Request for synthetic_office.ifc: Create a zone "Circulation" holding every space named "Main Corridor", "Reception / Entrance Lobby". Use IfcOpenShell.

First a look at what the model holds.

```python
import ifcopenshell

model = ifcopenshell.open("synthetic_office.ifc")
print(model.schema)
seen = {}
for space in model.by_type("IfcSpace"):
    seen[space.LongName] = seen.get(space.LongName, 0) + 1
for name, count in sorted(seen.items(), key=str):
    print(count, "x", name)
print("zones:", [z.Name for z in model.by_type("IfcZone")][:20])
```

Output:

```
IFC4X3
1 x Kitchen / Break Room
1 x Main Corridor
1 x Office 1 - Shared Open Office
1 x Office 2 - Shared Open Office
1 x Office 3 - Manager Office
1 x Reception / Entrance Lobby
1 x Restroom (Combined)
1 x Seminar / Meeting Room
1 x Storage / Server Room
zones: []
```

```python
import ifcopenshell
import ifcopenshell.api.group
import ifcopenshell.api.root

model = ifcopenshell.open("synthetic_office.ifc")

names = {"Main Corridor", "Reception / Entrance Lobby"}
spaces = [s for s in model.by_type("IfcSpace") if s.LongName in names]

zone = ifcopenshell.api.root.create_entity(model, ifc_class="IfcZone", name="Circulation")
ifcopenshell.api.group.assign_group(model, products=spaces, group=zone)
print(len(spaces), "spaces in", zone.Name)

model.write("synthetic_office_updated.ifc")
```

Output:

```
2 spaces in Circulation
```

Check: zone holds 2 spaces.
